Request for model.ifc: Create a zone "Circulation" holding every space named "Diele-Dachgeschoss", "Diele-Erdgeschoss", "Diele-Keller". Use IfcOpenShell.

First a look at what the model holds.

```python
import ifcopenshell

model = ifcopenshell.open("model.ifc")
print(model.schema)
seen = {}
for space in model.by_type("IfcSpace"):
    seen[space.LongName] = seen.get(space.LongName, 0) + 1
for name, count in sorted(seen.items(), key=str):
    print(count, "x", name)
print("zones:", [z.Name for z in model.by_type("IfcZone")][:20])
```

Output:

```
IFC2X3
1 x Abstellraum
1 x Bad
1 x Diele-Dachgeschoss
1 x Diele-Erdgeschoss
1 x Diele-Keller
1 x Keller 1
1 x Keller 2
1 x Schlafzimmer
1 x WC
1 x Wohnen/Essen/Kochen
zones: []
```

```python
import ifcopenshell
import ifcopenshell.api.group
import ifcopenshell.api.root

model = ifcopenshell.open("model.ifc")

names = {"Diele-Dachgeschoss", "Diele-Erdgeschoss", "Diele-Keller"}
spaces = [s for s in model.by_type("IfcSpace") if s.LongName in names]

zone = ifcopenshell.api.root.create_entity(model, ifc_class="IfcZone", name="Circulation")
ifcopenshell.api.group.assign_group(model, products=spaces, group=zone)
print(len(spaces), "spaces in", zone.Name)

model.write("model_v2.ifc")
```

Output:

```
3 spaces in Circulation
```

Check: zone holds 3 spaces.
